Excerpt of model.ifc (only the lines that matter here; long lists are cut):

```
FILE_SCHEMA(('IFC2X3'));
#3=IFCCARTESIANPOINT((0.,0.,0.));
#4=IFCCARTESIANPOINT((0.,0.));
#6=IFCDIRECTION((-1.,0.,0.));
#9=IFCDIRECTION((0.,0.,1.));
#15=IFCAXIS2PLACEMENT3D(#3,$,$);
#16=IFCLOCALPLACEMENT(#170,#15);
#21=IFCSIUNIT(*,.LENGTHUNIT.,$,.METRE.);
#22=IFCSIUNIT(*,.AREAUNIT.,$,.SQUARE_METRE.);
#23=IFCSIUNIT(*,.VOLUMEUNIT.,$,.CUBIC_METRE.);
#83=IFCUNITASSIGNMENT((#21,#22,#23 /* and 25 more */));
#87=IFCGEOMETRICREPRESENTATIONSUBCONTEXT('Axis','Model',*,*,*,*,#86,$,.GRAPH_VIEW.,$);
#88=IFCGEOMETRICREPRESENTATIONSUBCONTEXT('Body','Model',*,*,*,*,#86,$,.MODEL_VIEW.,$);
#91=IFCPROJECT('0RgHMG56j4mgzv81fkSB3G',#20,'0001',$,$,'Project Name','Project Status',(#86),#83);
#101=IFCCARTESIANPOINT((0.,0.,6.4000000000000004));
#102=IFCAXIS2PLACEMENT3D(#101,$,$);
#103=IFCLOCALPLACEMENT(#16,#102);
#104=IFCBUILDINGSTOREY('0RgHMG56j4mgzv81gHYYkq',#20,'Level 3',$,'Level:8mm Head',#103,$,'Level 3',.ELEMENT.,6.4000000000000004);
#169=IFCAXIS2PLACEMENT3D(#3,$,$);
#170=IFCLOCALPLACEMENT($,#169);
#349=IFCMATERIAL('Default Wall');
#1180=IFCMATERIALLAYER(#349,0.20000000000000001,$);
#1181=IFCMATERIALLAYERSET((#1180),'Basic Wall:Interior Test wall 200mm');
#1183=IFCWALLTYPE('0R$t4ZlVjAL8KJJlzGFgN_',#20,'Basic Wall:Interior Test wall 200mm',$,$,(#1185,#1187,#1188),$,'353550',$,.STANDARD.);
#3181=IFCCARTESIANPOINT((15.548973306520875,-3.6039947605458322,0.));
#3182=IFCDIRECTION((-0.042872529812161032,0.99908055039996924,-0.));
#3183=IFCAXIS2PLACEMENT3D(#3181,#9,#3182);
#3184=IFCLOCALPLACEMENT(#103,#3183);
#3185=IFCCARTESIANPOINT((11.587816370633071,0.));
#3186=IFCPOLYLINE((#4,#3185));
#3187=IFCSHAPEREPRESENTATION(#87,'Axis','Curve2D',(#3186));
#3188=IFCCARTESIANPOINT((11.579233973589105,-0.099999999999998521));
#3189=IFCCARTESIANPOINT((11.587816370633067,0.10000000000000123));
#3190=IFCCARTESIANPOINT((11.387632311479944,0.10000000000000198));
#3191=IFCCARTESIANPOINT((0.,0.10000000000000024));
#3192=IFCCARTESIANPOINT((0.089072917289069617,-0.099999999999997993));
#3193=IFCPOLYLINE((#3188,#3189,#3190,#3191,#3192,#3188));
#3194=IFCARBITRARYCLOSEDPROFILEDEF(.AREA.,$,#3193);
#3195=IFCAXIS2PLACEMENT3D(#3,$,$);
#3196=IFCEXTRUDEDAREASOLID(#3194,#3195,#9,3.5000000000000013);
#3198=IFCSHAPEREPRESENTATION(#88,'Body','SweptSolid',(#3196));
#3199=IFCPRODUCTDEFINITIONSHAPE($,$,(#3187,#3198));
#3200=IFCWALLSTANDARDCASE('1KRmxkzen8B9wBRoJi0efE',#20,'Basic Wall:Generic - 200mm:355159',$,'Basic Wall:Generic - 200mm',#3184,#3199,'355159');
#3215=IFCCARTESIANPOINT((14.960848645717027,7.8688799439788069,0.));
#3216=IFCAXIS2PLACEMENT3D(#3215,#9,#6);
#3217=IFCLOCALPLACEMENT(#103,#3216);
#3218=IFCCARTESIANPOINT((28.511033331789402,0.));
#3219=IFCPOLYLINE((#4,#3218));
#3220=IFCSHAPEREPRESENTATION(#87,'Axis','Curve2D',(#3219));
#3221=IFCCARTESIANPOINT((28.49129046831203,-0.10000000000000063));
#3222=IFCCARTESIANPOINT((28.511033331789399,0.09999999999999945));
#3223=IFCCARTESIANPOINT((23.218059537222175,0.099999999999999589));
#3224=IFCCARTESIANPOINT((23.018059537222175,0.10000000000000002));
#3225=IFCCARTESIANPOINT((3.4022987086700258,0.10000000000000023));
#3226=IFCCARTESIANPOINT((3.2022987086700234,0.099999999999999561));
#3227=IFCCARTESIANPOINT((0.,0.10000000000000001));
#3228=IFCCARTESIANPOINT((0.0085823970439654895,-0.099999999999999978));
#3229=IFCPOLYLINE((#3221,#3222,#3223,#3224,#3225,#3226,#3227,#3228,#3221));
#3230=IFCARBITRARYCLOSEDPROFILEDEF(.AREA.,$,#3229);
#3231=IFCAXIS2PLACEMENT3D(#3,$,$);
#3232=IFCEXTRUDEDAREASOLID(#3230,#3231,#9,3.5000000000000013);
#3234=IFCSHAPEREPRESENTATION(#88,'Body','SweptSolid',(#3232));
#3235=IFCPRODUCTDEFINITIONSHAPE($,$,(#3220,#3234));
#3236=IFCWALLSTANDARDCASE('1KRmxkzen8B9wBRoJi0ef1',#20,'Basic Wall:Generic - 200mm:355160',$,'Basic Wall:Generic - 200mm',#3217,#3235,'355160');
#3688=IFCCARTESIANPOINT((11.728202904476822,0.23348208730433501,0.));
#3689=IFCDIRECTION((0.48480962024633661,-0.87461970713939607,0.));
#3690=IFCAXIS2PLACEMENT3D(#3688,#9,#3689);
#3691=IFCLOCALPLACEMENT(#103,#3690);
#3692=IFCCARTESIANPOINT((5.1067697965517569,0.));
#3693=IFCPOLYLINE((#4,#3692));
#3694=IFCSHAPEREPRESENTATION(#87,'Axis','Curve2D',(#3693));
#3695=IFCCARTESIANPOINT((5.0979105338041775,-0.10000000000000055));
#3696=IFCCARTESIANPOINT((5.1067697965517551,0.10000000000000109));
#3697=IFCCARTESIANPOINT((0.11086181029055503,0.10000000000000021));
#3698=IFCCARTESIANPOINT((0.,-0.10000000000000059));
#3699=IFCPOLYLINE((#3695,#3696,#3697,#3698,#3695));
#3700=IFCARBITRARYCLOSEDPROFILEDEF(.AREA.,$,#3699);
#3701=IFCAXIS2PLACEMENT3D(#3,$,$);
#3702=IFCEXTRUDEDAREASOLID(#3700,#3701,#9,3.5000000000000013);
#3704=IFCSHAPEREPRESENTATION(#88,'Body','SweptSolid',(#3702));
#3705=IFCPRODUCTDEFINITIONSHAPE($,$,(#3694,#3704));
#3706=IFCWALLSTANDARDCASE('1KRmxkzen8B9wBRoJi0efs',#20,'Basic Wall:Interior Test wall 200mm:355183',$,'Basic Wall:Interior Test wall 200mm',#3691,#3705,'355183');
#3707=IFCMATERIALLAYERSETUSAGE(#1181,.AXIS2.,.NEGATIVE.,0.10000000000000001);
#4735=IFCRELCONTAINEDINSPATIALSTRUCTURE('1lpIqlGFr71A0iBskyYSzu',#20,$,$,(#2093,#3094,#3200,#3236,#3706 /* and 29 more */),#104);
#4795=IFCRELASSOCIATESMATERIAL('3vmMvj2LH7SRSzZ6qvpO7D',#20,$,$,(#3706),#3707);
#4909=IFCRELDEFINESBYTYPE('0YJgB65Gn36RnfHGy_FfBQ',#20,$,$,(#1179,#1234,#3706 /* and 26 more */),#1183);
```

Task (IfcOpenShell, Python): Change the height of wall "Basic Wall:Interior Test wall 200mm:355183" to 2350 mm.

```python
import ifcopenshell
import ifcopenshell.geom
import ifcopenshell.util.representation
import ifcopenshell.util.shape
import ifcopenshell.util.unit

model = ifcopenshell.open("model.ifc")
unit_scale = ifcopenshell.util.unit.calculate_unit_scale(model)
settings = ifcopenshell.geom.settings()


def volume(element):
    """Net volume in cubic metres, openings subtracted."""
    shape = ifcopenshell.geom.create_shape(settings, element)
    return ifcopenshell.util.shape.get_volume(shape.geometry)


wall = model.by_id(3706)
before = volume(wall)

body = ifcopenshell.util.representation.get_representation(wall, "Model", "Body")
solid = body.Items[0]
old_height = solid.Depth
solid.Depth = 2.35 / unit_scale
after = volume(wall)

print(f"height {old_height:g} -> {solid.Depth:g}, volume {before:.3f} -> {after:.3f} m3")

model.write("model_v2.ifc")
```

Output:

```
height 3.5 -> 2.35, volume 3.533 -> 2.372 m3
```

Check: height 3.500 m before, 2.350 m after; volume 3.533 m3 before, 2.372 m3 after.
